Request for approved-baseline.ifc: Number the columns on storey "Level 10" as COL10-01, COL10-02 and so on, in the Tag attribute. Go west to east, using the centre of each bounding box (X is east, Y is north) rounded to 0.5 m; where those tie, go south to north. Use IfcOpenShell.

First a look at what the model holds.

```python
import ifcopenshell
import ifcopenshell.util.element
import ifcopenshell.util.placement

model = ifcopenshell.open("approved-baseline.ifc")
print(model.schema)
storey = next(s for s in model.by_type("IfcBuildingStorey") if s.Name == "Level 10")
columns = [e for e in ifcopenshell.util.element.get_decomposition(storey) if e.is_a("IfcColumn")]
for e in sorted(columns, key=lambda e: e.id()):
    origin = ifcopenshell.util.placement.get_local_placement(e.ObjectPlacement)[:3, 3]
    print(e.id(), e.Tag, e.Name, origin.round(2) + 0.0, sep=" | ")
```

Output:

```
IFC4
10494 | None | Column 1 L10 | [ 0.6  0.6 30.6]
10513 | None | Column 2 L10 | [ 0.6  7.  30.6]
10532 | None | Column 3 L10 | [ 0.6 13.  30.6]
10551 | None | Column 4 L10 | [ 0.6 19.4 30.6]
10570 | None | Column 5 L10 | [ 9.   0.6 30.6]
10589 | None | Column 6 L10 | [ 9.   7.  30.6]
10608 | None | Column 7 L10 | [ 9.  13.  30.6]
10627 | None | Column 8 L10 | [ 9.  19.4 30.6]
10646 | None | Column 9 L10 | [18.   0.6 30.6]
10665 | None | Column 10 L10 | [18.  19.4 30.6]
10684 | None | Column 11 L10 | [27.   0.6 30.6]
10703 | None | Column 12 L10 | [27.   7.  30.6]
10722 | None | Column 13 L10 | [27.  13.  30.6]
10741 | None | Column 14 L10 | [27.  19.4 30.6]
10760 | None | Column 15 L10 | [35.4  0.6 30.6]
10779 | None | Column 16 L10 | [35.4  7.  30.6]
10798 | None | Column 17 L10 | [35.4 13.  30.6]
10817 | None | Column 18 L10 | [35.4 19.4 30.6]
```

```python
import ifcopenshell
import ifcopenshell.geom
import ifcopenshell.util.element
import ifcopenshell.util.shape

model = ifcopenshell.open("approved-baseline.ifc")
settings = ifcopenshell.geom.settings()
settings.set("use-world-coords", True)


def centre(element):
    shape = ifcopenshell.geom.create_shape(settings, element)
    return ifcopenshell.util.shape.get_bbox_centroid(shape.geometry)


storey = next(s for s in model.by_type("IfcBuildingStorey") if s.Name == "Level 10")
columns = [e for e in ifcopenshell.util.element.get_decomposition(storey) if e.is_a("IfcColumn")]

# Insertion points can sit at a corner or the storey origin, so sort by the geometry (in metres).
centres = {e: centre(e) for e in columns}
columns.sort(key=lambda e: (round(centres[e][0] / 0.5), centres[e][1]))

for i, e in enumerate(columns, start=1):
    number = f"COL10-{i:02d}"
    e.Tag = number
    print(e.id(), number)

model.write("approved-baseline_v2.ifc")
```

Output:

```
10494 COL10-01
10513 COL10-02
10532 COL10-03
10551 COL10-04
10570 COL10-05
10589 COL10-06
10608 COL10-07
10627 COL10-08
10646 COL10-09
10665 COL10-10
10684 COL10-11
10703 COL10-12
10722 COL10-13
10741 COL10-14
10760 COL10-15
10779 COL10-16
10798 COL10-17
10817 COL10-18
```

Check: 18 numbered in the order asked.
